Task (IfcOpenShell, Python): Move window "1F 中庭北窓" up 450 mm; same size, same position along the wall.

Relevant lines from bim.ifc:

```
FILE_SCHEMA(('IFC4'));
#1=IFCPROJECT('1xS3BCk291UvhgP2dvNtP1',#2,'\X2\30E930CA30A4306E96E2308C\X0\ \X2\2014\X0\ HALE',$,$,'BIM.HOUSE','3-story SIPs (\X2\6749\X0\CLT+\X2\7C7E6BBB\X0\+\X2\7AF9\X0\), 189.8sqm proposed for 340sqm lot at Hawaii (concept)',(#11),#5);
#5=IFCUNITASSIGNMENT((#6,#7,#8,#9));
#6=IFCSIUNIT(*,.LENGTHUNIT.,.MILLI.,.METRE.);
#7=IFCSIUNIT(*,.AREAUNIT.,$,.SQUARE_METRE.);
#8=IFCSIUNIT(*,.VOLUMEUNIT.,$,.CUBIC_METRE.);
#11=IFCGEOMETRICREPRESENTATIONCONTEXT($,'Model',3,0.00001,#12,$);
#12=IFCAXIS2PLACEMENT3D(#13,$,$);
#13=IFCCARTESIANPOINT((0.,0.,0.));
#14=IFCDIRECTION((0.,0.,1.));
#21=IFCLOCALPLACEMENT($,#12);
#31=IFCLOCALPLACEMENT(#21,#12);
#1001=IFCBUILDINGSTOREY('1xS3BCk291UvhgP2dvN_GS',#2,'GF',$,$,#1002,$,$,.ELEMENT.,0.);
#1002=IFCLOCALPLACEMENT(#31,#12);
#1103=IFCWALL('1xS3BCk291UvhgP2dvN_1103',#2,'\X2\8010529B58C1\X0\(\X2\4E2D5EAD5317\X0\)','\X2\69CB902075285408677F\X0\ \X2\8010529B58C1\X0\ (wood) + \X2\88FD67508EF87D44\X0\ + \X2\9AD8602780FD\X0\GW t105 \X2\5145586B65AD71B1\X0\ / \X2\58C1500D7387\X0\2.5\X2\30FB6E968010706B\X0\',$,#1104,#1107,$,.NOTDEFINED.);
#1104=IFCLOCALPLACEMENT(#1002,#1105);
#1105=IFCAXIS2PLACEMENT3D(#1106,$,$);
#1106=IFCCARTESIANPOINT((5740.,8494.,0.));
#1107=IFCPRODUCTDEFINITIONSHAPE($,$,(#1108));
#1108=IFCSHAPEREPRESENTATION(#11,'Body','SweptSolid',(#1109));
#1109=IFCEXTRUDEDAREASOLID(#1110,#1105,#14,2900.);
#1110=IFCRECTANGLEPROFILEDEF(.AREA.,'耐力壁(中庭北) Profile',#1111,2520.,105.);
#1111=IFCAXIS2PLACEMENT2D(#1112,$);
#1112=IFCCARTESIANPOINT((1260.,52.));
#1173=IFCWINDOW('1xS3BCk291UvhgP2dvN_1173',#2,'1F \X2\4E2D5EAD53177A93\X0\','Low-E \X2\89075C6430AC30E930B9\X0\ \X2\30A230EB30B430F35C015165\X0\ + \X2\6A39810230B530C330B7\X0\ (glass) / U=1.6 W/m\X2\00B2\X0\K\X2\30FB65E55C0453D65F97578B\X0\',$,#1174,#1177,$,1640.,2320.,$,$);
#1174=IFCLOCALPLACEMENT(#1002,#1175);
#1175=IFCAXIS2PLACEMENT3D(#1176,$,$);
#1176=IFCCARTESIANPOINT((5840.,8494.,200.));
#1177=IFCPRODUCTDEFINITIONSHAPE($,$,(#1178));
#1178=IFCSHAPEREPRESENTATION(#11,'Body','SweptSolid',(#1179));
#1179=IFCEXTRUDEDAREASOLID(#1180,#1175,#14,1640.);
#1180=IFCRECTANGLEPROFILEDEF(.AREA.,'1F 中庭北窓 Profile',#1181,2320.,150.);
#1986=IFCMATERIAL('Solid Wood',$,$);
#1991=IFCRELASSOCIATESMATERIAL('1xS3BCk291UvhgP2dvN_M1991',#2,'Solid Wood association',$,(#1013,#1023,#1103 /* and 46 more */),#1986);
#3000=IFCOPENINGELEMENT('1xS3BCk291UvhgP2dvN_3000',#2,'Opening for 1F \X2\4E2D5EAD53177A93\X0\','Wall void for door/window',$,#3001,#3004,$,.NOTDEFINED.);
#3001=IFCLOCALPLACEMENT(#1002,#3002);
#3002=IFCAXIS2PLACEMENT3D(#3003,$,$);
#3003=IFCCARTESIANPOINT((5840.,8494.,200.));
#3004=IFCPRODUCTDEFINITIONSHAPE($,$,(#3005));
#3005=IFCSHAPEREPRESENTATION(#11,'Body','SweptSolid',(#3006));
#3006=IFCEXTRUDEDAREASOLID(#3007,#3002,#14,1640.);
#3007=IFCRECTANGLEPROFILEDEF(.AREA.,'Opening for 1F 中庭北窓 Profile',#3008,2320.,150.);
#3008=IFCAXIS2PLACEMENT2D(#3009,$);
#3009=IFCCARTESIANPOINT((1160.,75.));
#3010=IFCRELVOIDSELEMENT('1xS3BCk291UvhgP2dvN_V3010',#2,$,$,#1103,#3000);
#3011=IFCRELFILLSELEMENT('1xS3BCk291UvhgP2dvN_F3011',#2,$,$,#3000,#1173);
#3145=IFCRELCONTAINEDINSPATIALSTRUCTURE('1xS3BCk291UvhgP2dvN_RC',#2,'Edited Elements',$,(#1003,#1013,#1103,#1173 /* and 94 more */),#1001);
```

```python
import numpy as np
import ifcopenshell
import ifcopenshell.api.geometry
import ifcopenshell.util.placement
import ifcopenshell.util.unit

model = ifcopenshell.open("bim.ifc")
unit_scale = ifcopenshell.util.unit.calculate_unit_scale(model)

window = model.by_id(1173)
opening = window.FillsVoids[0].RelatingOpeningElement
dz = 0.45 / unit_scale

shift = np.array([0.0, 0.0, dz])
# The window is not placed relative to its opening, so move both.
for product in (opening, window):
    matrix = ifcopenshell.util.placement.get_local_placement(product.ObjectPlacement)
    matrix[:3, 3] += shift
    ifcopenshell.api.geometry.edit_object_placement(model, product=product, matrix=matrix, is_si=False)

print(f"moved by {dz * unit_scale:+.3f} m")

model.write("bim_v2.ifc")
```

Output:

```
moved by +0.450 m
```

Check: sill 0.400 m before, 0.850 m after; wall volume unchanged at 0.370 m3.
